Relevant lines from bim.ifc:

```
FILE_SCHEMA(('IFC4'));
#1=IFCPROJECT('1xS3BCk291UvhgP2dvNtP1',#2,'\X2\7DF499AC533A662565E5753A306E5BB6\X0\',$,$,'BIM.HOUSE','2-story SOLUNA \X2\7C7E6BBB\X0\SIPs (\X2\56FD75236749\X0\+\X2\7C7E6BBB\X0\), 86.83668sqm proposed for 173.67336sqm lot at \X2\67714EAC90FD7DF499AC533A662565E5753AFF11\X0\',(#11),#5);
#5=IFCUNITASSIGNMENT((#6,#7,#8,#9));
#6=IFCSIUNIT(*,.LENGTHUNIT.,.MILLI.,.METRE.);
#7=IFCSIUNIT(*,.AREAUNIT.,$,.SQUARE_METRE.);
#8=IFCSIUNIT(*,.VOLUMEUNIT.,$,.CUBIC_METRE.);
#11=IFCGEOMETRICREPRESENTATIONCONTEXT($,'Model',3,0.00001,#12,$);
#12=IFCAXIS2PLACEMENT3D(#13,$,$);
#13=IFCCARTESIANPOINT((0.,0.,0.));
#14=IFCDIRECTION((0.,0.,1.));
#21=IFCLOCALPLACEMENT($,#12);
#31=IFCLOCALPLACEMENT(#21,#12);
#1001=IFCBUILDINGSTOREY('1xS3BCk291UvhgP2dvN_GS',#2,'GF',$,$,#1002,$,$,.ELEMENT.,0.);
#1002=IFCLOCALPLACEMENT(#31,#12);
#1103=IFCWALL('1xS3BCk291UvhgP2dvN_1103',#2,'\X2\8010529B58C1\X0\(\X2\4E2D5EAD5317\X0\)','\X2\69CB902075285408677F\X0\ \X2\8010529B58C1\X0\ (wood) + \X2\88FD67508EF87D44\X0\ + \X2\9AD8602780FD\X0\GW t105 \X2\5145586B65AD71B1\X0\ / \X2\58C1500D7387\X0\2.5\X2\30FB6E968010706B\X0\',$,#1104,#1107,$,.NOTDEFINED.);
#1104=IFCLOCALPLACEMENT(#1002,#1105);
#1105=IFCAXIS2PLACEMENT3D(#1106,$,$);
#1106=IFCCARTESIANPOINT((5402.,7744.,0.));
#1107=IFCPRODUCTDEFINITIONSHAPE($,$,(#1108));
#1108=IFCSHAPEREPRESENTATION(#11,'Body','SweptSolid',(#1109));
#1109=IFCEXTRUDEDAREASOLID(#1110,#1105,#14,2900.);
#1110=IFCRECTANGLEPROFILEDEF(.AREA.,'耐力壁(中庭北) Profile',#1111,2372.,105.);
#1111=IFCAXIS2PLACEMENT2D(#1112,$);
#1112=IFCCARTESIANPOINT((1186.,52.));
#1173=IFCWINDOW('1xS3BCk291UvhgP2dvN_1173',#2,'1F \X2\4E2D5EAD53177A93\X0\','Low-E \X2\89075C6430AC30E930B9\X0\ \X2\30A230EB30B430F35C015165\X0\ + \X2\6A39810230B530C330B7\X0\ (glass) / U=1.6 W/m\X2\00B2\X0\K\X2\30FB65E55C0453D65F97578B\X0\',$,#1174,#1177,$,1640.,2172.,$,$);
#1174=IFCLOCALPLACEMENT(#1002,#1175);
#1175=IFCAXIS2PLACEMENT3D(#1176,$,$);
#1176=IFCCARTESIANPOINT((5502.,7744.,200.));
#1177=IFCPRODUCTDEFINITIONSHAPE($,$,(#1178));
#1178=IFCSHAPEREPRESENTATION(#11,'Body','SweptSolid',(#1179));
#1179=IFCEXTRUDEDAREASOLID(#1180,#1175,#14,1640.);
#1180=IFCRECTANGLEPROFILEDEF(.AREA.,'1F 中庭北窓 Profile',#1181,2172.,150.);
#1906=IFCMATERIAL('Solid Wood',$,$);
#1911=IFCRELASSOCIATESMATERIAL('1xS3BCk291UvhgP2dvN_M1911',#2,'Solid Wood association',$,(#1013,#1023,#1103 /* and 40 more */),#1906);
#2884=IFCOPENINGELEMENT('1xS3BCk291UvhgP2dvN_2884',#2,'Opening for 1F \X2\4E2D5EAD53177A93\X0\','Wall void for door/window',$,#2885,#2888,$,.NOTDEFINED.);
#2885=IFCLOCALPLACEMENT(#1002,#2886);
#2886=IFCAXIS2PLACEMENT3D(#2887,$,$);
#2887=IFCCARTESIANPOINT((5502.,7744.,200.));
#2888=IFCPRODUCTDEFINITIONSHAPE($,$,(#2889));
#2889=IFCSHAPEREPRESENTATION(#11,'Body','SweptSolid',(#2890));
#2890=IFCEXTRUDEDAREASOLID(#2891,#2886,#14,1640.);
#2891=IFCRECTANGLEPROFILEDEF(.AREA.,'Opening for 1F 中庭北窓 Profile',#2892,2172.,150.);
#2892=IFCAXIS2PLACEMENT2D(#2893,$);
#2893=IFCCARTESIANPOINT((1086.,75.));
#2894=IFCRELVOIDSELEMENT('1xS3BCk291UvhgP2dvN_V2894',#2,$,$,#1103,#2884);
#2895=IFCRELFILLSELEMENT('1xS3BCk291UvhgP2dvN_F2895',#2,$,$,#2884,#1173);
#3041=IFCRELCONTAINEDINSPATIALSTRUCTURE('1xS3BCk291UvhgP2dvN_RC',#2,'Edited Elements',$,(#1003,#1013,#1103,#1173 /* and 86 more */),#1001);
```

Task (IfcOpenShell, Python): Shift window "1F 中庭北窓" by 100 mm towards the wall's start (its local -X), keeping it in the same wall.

```python
import ifcopenshell
import ifcopenshell.api.geometry
import ifcopenshell.util.placement
import ifcopenshell.util.unit

model = ifcopenshell.open("bim.ifc")
unit_scale = ifcopenshell.util.unit.calculate_unit_scale(model)

window = model.by_id(1173)
opening = window.FillsVoids[0].RelatingOpeningElement
wall = opening.VoidsElements[0].RelatingBuildingElement

wall_matrix = ifcopenshell.util.placement.get_local_placement(wall.ObjectPlacement)
shift = wall_matrix[:3, 0] * -0.1 / unit_scale
before = ifcopenshell.util.placement.get_local_placement(window.ObjectPlacement)[:3, 3].copy()

# The window is not placed relative to its opening, so move both.
for product in (opening, window):
    matrix = ifcopenshell.util.placement.get_local_placement(product.ObjectPlacement)
    matrix[:3, 3] += shift
    ifcopenshell.api.geometry.edit_object_placement(model, product=product, matrix=matrix, is_si=False)

after = ifcopenshell.util.placement.get_local_placement(window.ObjectPlacement)[:3, 3]
print("window moved by", (after - before).round(3) + 0.0)

model.write("bim_updated.ifc")
```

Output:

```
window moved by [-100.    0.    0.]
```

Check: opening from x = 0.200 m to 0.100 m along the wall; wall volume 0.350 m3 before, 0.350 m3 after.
